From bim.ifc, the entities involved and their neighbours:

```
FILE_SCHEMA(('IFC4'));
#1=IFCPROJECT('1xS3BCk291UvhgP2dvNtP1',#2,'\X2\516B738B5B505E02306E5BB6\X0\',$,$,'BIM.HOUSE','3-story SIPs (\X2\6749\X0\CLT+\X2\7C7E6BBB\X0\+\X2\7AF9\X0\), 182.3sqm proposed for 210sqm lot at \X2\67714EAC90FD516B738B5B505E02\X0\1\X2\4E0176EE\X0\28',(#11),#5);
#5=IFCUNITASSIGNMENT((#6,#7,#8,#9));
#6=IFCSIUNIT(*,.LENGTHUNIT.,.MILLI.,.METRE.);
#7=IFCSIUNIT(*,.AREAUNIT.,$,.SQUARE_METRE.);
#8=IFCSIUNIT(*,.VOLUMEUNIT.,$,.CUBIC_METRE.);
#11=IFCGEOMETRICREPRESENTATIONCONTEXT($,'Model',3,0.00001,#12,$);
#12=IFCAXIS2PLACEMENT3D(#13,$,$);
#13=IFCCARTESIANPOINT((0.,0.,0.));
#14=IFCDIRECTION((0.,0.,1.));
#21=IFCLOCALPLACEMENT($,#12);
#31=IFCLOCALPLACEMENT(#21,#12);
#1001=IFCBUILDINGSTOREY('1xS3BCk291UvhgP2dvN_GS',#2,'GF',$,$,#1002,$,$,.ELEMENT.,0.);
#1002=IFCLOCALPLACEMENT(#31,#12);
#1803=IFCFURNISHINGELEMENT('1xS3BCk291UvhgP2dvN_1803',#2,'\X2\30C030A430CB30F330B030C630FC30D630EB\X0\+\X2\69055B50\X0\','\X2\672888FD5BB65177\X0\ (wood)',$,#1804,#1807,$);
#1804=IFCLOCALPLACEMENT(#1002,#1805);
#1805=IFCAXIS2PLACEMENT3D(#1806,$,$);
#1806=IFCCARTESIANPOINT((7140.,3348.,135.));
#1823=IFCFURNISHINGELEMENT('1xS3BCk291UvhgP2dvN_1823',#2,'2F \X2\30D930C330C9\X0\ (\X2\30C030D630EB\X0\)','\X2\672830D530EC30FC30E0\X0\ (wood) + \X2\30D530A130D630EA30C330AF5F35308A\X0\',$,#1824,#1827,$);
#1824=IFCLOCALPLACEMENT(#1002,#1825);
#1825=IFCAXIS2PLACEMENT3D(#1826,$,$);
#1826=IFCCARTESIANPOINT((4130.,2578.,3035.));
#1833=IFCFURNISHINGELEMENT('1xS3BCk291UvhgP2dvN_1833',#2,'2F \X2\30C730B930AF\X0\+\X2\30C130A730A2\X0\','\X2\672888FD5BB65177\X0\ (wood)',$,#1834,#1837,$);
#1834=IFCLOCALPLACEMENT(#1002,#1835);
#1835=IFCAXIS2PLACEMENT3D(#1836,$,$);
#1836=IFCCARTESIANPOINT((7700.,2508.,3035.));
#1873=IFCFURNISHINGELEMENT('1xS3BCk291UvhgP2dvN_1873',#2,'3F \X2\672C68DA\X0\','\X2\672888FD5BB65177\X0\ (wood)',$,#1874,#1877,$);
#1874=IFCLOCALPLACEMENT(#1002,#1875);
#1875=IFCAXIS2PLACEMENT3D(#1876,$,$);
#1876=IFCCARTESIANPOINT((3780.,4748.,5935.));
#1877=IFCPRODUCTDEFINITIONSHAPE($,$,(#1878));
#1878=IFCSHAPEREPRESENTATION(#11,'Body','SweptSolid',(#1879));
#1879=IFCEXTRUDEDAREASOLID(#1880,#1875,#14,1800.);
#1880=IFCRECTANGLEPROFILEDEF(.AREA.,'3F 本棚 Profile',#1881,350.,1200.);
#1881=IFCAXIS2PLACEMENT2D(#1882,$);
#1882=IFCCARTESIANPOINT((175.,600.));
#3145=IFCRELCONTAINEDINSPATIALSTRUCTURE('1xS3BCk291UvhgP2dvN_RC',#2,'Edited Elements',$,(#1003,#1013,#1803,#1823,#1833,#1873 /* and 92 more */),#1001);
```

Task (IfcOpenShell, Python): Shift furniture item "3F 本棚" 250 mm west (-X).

```python
import ifcopenshell
import ifcopenshell.api.geometry
import ifcopenshell.util.placement
import ifcopenshell.util.unit

model = ifcopenshell.open("bim.ifc")
unit_scale = ifcopenshell.util.unit.calculate_unit_scale(model)

item = model.by_id(1873)
matrix = ifcopenshell.util.placement.get_local_placement(item.ObjectPlacement)
matrix[0, 3] -= 0.25 / unit_scale
ifcopenshell.api.geometry.edit_object_placement(model, product=item, matrix=matrix, is_si=False)

print(ifcopenshell.util.placement.get_local_placement(item.ObjectPlacement).round(3) + 0.0)

model.write("bim_v2.ifc")
```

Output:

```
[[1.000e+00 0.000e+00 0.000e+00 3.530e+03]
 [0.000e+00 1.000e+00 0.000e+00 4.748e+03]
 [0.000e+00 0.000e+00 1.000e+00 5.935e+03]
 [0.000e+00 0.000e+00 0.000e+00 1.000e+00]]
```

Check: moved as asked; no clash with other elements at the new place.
